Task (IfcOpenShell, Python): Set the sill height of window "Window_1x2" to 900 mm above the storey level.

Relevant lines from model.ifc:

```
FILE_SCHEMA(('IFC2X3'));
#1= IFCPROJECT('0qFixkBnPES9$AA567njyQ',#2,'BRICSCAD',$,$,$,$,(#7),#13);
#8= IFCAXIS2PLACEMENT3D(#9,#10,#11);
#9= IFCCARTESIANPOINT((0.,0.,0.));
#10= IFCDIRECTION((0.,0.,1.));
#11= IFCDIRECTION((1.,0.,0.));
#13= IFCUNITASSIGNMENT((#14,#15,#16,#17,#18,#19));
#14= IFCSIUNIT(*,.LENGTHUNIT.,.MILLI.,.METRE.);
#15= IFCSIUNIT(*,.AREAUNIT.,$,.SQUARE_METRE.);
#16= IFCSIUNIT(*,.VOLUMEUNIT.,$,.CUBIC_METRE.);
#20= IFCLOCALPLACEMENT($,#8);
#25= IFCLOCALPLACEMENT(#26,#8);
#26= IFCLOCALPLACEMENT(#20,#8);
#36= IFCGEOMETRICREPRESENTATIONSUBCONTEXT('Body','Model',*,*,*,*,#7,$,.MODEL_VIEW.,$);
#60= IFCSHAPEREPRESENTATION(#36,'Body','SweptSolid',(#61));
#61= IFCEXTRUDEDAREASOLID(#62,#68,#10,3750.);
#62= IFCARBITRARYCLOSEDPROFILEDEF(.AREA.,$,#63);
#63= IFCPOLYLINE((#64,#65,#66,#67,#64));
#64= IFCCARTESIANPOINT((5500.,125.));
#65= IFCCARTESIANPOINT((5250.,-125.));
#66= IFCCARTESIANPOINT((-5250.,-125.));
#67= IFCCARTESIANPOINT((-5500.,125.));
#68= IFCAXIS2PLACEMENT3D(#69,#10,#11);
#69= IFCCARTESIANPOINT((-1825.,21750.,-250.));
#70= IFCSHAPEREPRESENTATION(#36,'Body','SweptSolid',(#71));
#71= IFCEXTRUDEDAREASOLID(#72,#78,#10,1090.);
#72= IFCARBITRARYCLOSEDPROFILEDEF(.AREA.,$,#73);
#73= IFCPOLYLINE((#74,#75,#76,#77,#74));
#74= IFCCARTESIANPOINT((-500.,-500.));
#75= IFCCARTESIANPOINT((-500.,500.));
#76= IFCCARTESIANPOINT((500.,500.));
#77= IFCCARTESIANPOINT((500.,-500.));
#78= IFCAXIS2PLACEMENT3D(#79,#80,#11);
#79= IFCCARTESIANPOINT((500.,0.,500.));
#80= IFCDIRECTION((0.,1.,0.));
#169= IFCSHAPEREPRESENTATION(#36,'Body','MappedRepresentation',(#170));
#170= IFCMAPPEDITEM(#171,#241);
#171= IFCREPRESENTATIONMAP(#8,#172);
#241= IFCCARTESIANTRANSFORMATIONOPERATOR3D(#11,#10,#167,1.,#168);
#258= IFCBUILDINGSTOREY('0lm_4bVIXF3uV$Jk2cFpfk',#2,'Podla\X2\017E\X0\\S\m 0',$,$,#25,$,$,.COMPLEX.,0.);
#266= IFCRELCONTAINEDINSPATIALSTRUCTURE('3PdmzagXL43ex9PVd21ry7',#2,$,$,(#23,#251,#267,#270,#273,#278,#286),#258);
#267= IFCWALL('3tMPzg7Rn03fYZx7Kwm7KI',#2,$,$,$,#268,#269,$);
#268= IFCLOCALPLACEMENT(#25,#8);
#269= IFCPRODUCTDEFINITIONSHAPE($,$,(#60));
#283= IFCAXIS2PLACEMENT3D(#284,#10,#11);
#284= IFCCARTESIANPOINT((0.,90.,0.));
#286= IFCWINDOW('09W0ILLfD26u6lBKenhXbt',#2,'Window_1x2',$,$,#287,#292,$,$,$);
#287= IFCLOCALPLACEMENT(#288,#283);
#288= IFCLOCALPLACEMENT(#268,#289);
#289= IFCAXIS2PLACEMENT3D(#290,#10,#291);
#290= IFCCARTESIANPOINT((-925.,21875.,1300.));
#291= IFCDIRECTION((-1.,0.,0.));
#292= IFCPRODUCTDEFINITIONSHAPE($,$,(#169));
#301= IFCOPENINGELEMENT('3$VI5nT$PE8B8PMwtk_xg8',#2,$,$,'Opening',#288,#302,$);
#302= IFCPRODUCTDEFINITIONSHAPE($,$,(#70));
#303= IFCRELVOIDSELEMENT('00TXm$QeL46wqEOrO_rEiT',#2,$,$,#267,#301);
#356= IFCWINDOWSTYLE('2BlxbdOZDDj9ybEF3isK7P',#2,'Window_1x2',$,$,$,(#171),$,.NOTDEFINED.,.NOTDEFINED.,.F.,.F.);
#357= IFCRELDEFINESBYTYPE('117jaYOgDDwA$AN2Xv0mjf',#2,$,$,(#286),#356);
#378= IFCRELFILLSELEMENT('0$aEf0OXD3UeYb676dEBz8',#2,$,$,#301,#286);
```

```python
import numpy as np
import ifcopenshell
import ifcopenshell.api.geometry
import ifcopenshell.geom
import ifcopenshell.util.element
import ifcopenshell.util.placement
import ifcopenshell.util.shape
import ifcopenshell.util.unit

model = ifcopenshell.open("model.ifc")
unit_scale = ifcopenshell.util.unit.calculate_unit_scale(model)

window = model.by_guid("09W0ILLfD26u6lBKenhXbt")
opening = window.FillsVoids[0].RelatingOpeningElement
storey = ifcopenshell.util.element.get_container(window, ifc_class="IfcBuildingStorey")
level = ifcopenshell.util.placement.get_local_placement(storey.ObjectPlacement)[2, 3]

# The opening's origin need not be at the sill, so measure its lowest point.
shape = ifcopenshell.geom.create_shape(ifcopenshell.geom.settings(), opening)
bottom = ifcopenshell.util.shape.get_shape_bottom_elevation(shape, shape.geometry) / unit_scale
dz = level + 0.9 / unit_scale - bottom

shift = np.array([0.0, 0.0, dz])
# The window is placed relative to its opening, so it follows when the opening moves.
matrix = ifcopenshell.util.placement.get_local_placement(opening.ObjectPlacement)
matrix[:3, 3] += shift
ifcopenshell.api.geometry.edit_object_placement(
    model, product=opening, matrix=matrix, is_si=False, should_transform_children=True
)

print(f"moved by {dz * unit_scale:+.3f} m")

model.write("model_updated.ifc")
```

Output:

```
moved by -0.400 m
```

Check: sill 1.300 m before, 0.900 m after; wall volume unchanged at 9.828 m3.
